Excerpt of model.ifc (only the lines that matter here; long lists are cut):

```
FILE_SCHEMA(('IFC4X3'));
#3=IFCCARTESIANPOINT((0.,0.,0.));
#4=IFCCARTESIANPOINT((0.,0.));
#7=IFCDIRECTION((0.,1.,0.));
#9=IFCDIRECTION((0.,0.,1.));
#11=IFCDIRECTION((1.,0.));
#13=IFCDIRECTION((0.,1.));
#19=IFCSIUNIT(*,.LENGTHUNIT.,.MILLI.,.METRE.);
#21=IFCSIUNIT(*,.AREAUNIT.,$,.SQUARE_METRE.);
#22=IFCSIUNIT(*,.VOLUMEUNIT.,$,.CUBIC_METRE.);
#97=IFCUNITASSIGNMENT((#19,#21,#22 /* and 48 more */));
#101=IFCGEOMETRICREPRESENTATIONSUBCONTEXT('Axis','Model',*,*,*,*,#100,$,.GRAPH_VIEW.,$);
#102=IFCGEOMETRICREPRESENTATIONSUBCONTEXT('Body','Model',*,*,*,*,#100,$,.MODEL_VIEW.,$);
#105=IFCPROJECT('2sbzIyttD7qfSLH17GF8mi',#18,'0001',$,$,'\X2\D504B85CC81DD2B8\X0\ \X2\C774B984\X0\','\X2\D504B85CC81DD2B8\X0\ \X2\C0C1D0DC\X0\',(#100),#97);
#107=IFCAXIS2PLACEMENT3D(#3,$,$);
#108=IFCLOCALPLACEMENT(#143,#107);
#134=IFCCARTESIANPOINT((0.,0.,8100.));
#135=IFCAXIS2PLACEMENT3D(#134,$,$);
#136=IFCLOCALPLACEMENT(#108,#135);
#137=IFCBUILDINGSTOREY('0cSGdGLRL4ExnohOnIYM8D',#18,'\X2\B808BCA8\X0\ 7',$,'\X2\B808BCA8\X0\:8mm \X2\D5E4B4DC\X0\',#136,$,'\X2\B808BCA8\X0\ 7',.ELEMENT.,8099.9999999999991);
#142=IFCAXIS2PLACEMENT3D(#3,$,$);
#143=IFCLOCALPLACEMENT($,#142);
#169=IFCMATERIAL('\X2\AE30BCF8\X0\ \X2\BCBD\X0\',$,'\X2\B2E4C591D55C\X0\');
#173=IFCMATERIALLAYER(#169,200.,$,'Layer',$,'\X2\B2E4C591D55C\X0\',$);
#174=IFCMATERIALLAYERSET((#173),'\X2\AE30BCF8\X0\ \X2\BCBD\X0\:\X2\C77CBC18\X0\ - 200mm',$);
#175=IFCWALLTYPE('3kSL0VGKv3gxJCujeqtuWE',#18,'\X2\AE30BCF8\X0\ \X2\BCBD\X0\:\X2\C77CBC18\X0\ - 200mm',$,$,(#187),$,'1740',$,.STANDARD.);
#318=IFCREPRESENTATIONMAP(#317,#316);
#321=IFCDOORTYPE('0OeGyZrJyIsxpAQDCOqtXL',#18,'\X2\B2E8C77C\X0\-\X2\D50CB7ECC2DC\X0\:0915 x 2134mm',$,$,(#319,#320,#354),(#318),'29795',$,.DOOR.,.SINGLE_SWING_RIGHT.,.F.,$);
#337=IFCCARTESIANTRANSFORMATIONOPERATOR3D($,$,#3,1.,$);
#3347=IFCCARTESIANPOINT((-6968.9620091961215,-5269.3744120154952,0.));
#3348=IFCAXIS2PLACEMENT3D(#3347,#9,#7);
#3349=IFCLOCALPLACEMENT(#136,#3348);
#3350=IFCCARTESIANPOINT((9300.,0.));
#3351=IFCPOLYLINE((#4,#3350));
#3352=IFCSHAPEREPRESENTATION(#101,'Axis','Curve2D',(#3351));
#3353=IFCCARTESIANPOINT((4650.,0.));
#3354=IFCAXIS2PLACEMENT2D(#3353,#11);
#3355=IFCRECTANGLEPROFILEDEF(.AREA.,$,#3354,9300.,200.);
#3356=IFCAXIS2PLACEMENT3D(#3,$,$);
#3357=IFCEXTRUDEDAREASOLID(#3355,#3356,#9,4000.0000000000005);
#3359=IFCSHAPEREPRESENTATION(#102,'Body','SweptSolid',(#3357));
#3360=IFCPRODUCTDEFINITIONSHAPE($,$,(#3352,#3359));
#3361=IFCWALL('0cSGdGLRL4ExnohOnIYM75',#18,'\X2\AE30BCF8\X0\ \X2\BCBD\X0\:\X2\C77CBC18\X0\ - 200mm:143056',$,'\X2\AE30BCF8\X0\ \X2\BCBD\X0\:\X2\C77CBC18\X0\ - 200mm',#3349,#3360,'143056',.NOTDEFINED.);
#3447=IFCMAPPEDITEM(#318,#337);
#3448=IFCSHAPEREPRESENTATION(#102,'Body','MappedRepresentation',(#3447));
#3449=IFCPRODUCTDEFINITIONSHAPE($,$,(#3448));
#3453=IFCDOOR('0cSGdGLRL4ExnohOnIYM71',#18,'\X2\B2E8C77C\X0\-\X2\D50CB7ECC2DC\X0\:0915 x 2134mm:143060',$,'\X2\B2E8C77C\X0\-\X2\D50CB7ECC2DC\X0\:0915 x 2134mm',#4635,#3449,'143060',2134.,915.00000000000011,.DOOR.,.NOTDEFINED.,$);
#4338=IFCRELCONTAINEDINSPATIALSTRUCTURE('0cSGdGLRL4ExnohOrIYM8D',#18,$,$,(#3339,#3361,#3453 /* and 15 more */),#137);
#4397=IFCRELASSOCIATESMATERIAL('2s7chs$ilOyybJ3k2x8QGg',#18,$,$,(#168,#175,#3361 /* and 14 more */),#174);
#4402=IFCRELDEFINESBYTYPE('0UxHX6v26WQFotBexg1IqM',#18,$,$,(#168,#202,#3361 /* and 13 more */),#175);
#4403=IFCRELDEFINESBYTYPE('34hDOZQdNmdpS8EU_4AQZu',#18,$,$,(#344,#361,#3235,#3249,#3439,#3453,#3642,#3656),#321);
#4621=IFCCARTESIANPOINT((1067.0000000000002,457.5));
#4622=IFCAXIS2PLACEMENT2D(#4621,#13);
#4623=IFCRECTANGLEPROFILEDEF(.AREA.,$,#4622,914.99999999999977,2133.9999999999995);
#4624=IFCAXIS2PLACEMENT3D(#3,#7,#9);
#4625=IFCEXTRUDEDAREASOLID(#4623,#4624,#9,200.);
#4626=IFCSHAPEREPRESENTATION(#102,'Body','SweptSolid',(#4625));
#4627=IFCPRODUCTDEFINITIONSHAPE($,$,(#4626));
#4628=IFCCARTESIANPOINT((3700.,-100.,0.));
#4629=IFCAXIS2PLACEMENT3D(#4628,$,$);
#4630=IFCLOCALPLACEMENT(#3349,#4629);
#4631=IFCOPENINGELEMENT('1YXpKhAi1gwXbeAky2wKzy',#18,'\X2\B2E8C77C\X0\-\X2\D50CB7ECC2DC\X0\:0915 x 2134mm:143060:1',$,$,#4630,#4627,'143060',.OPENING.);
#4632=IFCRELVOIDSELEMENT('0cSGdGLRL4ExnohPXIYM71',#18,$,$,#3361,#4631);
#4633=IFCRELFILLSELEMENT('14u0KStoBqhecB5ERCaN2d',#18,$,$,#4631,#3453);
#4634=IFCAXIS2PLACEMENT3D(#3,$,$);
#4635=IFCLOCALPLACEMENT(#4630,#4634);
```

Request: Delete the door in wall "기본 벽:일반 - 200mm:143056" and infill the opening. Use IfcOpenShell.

```python
import ifcopenshell
import ifcopenshell.api.feature
import ifcopenshell.api.root
import ifcopenshell.geom
import ifcopenshell.util.shape

model = ifcopenshell.open("model.ifc")
settings = ifcopenshell.geom.settings()


def volume(element):
    """Net volume in cubic metres, openings subtracted."""
    shape = ifcopenshell.geom.create_shape(settings, element)
    return ifcopenshell.util.shape.get_volume(shape.geometry)


door = model.by_guid("0cSGdGLRL4ExnohOnIYM71")
opening = door.FillsVoids[0].RelatingOpeningElement
wall = opening.VoidsElements[0].RelatingBuildingElement
before = volume(wall)

ifcopenshell.api.root.remove_product(model, product=door)
ifcopenshell.api.feature.remove_feature(model, feature=opening)

after = volume(wall)

print(f"wall volume {before:.3f} -> {after:.3f} m3")

model.write("model_updated.ifc")
```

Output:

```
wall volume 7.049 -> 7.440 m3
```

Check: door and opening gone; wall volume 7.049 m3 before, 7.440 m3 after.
